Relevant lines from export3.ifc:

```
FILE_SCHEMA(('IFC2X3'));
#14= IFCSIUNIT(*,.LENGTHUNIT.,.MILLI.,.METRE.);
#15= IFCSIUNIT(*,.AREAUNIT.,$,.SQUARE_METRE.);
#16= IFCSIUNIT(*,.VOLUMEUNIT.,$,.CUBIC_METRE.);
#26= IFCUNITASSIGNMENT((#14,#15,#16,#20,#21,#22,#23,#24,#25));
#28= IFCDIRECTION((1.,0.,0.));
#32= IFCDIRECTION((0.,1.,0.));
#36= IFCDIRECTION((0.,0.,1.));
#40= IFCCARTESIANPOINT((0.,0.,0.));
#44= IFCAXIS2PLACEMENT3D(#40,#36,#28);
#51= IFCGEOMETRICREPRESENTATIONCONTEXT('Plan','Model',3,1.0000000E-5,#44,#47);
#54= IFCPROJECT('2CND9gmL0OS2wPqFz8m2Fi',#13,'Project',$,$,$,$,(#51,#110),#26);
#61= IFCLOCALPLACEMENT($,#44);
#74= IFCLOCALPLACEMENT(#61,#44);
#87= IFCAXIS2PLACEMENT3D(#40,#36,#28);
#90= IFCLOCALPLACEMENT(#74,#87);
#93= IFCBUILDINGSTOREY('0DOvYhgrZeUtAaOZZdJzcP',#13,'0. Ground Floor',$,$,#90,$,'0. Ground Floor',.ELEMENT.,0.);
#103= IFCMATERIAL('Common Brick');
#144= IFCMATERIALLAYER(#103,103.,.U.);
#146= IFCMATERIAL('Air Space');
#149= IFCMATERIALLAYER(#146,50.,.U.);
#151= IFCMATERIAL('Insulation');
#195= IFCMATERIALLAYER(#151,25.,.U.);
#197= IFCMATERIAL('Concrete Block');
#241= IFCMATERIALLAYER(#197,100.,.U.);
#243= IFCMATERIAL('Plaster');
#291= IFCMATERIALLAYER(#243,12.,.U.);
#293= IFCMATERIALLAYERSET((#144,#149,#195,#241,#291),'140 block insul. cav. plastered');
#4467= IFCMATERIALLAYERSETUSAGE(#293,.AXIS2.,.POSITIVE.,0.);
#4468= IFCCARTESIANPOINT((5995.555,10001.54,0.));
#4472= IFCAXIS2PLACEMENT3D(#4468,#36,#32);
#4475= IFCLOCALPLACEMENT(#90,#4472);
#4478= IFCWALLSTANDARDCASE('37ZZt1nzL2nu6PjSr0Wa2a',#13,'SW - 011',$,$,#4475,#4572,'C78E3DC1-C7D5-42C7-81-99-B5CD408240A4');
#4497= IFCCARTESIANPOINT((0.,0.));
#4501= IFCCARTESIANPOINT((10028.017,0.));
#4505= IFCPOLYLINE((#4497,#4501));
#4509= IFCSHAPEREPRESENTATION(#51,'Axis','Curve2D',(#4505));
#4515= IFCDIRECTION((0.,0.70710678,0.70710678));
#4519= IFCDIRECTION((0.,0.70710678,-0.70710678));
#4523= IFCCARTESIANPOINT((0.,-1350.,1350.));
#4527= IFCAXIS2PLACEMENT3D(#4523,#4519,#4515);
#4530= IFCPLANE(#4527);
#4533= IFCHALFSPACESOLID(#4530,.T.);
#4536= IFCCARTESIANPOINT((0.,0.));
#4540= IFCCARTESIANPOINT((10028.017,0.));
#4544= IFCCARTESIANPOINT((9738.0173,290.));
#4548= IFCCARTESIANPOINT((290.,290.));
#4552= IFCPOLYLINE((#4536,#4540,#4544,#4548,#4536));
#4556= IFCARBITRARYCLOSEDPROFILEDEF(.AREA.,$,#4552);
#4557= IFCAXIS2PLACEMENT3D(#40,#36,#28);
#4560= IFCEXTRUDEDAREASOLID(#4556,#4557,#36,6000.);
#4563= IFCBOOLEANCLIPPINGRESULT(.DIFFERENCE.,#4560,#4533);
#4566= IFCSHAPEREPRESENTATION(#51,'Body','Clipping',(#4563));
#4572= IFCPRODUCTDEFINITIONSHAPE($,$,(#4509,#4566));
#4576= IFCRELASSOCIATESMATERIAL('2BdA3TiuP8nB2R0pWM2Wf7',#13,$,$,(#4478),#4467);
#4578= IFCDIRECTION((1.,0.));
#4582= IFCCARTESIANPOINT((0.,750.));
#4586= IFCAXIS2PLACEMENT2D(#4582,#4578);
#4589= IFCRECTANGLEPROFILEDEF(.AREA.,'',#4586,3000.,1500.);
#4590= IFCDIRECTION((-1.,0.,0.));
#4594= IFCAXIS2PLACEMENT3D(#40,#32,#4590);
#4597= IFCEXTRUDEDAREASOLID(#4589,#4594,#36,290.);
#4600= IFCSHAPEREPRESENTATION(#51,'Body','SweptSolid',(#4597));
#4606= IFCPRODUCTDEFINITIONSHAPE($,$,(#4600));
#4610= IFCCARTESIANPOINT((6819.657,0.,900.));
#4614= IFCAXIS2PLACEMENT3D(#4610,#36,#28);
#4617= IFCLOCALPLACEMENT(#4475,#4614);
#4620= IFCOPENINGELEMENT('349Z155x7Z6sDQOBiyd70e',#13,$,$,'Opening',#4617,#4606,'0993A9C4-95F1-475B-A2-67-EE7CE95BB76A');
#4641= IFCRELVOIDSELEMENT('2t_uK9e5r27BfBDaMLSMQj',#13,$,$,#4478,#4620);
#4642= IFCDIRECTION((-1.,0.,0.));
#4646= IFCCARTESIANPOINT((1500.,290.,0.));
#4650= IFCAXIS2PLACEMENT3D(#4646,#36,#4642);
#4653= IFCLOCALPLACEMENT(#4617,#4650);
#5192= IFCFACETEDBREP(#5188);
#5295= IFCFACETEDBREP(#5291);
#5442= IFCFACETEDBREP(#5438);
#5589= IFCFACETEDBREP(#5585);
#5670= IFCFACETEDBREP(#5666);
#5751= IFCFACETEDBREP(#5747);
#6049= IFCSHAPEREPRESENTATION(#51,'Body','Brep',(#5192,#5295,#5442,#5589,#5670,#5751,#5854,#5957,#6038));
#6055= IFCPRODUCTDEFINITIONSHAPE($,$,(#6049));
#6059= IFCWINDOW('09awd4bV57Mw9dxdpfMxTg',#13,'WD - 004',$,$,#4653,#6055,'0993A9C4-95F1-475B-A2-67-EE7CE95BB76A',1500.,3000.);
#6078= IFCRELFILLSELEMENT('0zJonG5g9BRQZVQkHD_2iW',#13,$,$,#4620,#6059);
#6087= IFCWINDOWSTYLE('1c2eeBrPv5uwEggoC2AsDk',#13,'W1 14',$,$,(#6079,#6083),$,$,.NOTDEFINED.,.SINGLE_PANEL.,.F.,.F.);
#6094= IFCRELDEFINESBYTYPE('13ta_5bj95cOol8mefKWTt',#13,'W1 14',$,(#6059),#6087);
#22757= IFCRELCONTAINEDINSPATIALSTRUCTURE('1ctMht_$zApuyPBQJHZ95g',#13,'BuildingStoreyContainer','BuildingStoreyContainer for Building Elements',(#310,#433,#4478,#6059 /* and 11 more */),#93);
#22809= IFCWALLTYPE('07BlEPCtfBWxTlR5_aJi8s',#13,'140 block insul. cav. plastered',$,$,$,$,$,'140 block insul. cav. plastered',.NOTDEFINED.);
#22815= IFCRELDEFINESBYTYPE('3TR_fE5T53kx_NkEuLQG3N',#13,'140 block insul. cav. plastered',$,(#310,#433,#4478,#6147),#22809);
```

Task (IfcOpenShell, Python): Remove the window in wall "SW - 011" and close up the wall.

```python
import ifcopenshell
import ifcopenshell.api.feature
import ifcopenshell.api.root
import ifcopenshell.geom
import ifcopenshell.util.shape

model = ifcopenshell.open("export3.ifc")
settings = ifcopenshell.geom.settings()


def volume(element):
    """Net volume in cubic metres, openings subtracted."""
    shape = ifcopenshell.geom.create_shape(settings, element)
    return ifcopenshell.util.shape.get_volume(shape.geometry)


window = model.by_guid("09awd4bV57Mw9dxdpfMxTg")
opening = window.FillsVoids[0].RelatingOpeningElement
wall = opening.VoidsElements[0].RelatingBuildingElement
before = volume(wall)

ifcopenshell.api.root.remove_product(model, product=window)
ifcopenshell.api.feature.remove_feature(model, feature=opening)

after = volume(wall)

print(f"wall volume {before:.3f} -> {after:.3f} m3")

model.write("export3_updated.ifc")
```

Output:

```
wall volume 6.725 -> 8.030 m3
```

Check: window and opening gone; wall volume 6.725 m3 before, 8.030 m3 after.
